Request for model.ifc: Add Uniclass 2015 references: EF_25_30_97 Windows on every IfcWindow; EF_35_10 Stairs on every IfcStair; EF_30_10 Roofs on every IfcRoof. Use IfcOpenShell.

First a look at what the model holds.

```python
import ifcopenshell

model = ifcopenshell.open("model.ifc")
print(model.schema)
print("classifications:", [c.Name for c in model.by_type("IfcClassification")])
for ifc_class in ("IfcDoor", "IfcRoof", "IfcStair", "IfcWall", "IfcWindow"):
    print(ifc_class, len(model.by_type(ifc_class)))
```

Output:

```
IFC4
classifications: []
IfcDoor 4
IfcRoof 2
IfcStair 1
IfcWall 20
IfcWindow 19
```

```python
import ifcopenshell
import ifcopenshell.api.classification

model = ifcopenshell.open("model.ifc")

system = ifcopenshell.api.classification.add_classification(model, classification="Uniclass 2015")

codes = {
    "IfcWindow": ("EF_25_30_97", "Windows"),
    "IfcStair": ("EF_35_10", "Stairs"),
    "IfcRoof": ("EF_30_10", "Roofs"),
}
for ifc_class, (code, name) in codes.items():
    products = model.by_type(ifc_class)
    ifcopenshell.api.classification.add_reference(
        model, products=products, classification=system, identification=code, name=name
    )
    print(code, len(products))

model.write("model_updated.ifc")
```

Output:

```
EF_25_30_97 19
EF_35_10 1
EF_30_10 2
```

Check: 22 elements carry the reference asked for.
